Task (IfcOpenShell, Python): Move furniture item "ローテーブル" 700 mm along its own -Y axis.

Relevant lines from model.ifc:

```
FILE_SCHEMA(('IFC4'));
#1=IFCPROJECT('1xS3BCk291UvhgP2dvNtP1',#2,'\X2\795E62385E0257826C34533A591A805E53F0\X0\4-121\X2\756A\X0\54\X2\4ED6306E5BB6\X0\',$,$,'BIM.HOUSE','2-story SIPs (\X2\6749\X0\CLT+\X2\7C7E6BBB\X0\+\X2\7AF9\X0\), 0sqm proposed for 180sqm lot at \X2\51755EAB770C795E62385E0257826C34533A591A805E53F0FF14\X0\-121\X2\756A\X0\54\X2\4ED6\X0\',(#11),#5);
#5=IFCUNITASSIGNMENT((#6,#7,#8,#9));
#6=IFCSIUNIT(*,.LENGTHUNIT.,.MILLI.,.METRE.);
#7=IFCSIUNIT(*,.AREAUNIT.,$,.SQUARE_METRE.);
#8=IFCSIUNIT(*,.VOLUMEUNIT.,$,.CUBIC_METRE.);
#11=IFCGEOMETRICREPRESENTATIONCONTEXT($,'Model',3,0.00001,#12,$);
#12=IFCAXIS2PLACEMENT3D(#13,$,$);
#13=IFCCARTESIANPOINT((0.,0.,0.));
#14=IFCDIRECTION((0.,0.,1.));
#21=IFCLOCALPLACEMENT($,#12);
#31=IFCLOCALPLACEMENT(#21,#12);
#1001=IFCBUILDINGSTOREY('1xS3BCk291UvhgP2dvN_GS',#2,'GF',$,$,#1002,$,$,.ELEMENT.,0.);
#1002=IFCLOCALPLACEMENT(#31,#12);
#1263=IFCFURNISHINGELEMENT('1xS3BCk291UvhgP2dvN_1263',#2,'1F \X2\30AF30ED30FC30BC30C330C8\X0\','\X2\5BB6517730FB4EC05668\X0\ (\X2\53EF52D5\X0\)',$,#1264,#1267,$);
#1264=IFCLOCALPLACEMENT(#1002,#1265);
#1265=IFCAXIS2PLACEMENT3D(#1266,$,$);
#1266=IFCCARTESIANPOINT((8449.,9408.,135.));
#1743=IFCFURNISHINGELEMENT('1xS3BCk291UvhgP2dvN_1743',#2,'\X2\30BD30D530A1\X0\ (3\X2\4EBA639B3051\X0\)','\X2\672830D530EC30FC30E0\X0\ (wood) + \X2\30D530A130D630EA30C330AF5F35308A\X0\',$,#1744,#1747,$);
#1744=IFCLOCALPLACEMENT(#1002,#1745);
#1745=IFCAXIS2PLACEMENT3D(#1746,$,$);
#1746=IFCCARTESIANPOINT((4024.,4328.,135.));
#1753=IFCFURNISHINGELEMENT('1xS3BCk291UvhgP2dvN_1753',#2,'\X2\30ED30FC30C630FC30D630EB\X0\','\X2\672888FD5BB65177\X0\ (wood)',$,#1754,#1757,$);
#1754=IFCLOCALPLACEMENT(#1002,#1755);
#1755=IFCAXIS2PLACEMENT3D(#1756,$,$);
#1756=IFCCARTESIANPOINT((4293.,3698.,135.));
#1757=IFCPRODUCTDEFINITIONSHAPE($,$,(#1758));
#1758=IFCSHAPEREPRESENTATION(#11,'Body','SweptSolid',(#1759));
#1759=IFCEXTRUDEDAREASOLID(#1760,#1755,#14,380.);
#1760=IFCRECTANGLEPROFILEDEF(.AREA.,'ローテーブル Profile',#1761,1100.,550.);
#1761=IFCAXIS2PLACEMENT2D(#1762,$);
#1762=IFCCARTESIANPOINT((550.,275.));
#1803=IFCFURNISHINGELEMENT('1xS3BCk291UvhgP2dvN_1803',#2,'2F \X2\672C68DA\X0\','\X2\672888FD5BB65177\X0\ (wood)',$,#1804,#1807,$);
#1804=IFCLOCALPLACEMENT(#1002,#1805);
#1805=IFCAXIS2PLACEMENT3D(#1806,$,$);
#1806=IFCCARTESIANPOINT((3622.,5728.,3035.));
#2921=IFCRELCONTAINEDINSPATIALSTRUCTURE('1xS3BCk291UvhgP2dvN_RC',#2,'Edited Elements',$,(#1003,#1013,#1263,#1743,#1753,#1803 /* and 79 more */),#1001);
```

```python
import ifcopenshell
import ifcopenshell.api.geometry
import ifcopenshell.util.placement

model = ifcopenshell.open("model.ifc")

item = model.by_guid("1xS3BCk291UvhgP2dvN_1753")
matrix = ifcopenshell.util.placement.get_local_placement(item.ObjectPlacement)
matrix[:3, 3] -= matrix[:3, 1] * 700.0
ifcopenshell.api.geometry.edit_object_placement(model, product=item, matrix=matrix, is_si=False)

print(ifcopenshell.util.placement.get_local_placement(item.ObjectPlacement).round(3) + 0.0)

model.write("model_v2.ifc")
```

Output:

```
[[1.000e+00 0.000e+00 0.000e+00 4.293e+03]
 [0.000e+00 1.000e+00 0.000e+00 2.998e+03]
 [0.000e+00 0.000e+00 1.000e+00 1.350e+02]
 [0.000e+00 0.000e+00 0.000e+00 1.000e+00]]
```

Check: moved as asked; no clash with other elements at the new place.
